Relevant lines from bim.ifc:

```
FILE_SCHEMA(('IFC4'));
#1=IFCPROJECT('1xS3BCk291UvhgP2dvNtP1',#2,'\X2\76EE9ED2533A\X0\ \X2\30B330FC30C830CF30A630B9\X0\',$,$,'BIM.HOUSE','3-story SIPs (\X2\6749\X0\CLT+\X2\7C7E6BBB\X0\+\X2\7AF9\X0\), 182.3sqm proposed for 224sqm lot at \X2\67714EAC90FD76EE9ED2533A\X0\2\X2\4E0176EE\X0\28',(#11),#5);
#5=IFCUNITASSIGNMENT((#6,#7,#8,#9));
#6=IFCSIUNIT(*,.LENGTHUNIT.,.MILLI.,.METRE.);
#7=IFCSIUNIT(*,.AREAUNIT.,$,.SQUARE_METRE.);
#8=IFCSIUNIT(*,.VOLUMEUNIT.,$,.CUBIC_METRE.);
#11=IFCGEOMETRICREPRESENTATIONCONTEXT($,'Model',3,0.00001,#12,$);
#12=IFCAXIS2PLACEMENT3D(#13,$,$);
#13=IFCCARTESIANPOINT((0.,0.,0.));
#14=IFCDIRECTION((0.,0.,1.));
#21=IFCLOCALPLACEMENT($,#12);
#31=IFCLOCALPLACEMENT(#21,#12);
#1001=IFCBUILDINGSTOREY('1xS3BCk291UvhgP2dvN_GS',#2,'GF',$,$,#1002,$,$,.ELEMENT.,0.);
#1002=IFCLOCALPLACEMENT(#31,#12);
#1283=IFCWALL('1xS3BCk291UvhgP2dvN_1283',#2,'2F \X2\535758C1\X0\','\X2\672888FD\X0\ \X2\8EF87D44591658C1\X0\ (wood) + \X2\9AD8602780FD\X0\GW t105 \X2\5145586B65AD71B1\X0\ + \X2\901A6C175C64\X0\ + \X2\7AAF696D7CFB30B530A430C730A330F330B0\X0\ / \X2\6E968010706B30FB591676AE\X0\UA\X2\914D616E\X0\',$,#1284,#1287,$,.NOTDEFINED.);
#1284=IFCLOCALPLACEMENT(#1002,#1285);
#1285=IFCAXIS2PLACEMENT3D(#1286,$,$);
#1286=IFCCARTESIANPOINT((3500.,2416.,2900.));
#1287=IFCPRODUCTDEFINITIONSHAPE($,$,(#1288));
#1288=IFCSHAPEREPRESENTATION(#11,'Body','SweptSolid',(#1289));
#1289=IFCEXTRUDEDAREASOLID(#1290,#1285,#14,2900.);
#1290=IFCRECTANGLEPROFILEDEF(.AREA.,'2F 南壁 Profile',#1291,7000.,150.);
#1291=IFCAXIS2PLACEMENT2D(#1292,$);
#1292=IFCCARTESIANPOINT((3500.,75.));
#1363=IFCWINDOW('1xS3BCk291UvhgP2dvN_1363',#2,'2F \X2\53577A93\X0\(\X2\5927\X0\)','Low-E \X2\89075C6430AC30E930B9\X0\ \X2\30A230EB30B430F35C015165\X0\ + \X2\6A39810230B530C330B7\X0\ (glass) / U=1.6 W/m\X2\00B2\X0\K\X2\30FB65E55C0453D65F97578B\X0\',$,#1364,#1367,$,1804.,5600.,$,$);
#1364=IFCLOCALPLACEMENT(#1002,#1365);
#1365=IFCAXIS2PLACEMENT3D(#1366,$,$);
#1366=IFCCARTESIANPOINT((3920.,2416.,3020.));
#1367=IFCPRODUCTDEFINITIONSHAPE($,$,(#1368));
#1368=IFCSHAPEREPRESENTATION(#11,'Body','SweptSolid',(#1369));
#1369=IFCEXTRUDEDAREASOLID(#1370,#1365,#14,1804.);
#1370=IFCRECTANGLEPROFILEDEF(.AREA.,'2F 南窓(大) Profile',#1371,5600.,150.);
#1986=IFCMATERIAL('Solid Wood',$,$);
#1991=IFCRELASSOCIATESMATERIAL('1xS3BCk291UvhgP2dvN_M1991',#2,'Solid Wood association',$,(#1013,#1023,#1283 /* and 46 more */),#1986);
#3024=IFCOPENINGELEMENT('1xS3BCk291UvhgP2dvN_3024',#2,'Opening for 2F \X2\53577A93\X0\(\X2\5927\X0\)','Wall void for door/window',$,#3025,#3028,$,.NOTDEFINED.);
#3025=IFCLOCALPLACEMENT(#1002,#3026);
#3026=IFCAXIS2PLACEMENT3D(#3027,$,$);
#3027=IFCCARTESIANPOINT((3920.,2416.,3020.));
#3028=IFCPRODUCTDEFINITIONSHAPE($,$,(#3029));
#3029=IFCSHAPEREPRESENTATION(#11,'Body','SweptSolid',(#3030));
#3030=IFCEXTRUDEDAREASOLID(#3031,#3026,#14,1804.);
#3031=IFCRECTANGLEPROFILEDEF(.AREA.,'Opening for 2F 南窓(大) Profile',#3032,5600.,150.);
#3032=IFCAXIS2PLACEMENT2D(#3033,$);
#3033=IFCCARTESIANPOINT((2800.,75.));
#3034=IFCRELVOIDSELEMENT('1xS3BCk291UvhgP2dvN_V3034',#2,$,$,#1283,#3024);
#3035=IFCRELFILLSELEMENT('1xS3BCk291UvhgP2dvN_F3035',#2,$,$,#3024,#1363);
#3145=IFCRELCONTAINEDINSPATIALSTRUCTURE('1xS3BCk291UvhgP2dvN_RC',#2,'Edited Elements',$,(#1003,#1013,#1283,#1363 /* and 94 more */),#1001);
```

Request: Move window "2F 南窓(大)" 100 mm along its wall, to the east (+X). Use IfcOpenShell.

```python
import ifcopenshell
import ifcopenshell.api.geometry
import ifcopenshell.util.placement

model = ifcopenshell.open("bim.ifc")

window = model.by_id(1363)
opening = window.FillsVoids[0].RelatingOpeningElement
wall = opening.VoidsElements[0].RelatingBuildingElement

wall_matrix = ifcopenshell.util.placement.get_local_placement(wall.ObjectPlacement)
shift = wall_matrix[:3, 0] * 100.0
before = ifcopenshell.util.placement.get_local_placement(window.ObjectPlacement)[:3, 3].copy()

# The window is not placed relative to its opening, so move both.
for product in (opening, window):
    matrix = ifcopenshell.util.placement.get_local_placement(product.ObjectPlacement)
    matrix[:3, 3] += shift
    ifcopenshell.api.geometry.edit_object_placement(model, product=product, matrix=matrix, is_si=False)

after = ifcopenshell.util.placement.get_local_placement(window.ObjectPlacement)[:3, 3]
print("window moved by", (after - before).round(3) + 0.0)

model.write("bim_v2.ifc")
```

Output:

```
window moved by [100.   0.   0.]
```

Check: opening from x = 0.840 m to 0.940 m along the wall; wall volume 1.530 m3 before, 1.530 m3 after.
